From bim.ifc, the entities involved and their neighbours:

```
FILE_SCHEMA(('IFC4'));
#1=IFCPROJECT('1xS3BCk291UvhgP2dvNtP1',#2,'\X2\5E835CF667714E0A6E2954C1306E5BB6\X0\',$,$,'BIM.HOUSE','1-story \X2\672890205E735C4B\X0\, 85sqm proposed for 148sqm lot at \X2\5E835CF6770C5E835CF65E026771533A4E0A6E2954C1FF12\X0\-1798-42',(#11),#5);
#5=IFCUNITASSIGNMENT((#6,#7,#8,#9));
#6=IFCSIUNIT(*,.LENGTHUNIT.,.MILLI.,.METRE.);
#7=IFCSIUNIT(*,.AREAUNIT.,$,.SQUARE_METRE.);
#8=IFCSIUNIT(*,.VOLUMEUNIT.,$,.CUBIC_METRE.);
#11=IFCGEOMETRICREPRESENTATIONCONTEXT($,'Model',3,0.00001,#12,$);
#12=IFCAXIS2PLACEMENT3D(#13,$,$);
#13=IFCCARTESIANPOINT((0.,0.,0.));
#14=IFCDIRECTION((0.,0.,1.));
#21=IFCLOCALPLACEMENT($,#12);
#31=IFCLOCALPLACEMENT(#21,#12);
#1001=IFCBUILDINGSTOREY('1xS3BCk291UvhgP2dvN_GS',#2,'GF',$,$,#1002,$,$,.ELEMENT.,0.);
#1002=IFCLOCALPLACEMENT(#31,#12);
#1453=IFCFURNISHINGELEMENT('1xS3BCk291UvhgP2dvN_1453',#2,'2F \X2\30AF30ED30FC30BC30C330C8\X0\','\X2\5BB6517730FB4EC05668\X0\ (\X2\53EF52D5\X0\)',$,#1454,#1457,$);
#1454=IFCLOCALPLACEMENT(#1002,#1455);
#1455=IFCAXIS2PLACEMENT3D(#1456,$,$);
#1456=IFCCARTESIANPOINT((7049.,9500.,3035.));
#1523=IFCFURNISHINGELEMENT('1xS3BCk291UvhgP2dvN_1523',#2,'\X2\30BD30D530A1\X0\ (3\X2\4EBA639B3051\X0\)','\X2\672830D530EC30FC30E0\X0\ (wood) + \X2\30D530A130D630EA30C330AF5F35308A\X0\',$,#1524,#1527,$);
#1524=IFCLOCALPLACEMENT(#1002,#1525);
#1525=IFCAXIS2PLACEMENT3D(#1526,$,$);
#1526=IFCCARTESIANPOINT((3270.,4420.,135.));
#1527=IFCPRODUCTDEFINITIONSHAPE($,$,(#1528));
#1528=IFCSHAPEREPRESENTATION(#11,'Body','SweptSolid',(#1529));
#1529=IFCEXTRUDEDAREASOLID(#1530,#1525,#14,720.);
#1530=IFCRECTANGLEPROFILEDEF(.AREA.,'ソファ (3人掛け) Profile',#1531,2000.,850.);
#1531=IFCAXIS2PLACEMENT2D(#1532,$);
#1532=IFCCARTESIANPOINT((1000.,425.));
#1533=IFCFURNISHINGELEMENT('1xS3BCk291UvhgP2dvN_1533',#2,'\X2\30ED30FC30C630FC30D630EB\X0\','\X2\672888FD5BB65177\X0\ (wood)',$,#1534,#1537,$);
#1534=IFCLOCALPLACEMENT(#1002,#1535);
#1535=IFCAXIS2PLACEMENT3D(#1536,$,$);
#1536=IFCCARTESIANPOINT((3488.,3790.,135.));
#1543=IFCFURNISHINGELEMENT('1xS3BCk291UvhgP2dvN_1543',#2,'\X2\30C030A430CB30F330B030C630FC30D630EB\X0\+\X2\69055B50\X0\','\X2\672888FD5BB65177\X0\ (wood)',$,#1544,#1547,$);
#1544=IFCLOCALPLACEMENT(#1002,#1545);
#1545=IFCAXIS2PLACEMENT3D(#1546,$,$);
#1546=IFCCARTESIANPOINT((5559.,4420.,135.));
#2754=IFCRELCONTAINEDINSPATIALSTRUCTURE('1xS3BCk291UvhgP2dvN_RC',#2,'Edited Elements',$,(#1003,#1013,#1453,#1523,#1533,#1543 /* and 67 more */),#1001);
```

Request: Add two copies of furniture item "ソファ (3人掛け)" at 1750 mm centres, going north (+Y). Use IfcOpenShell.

```python
import numpy as np
import ifcopenshell
import ifcopenshell.api.geometry
import ifcopenshell.api.root
import ifcopenshell.util.element
import ifcopenshell.util.placement

model = ifcopenshell.open("bim.ifc")


def reuse_history(source, copy):
    """copy_class also copies each property set's owner history, people and application; keep the originals."""
    for rel in copy.IsDefinedBy:
        if rel.is_a("IfcRelDefinesByProperties") and (history := rel.RelatingPropertyDefinition.OwnerHistory):
            rel.RelatingPropertyDefinition.OwnerHistory = source.OwnerHistory
            ifcopenshell.util.element.remove_deep2(model, history)


source = model.by_guid("1xS3BCk291UvhgP2dvN_1523")
base = ifcopenshell.util.placement.get_local_placement(source.ObjectPlacement)
step = np.array([0.0, 1.0, 0.0]) * 1750.0

for i in range(1, 3):
    copy = ifcopenshell.api.root.copy_class(model, product=source)
    copy.Representation = ifcopenshell.util.element.copy_deep(
        model, source.Representation, exclude=["IfcGeometricRepresentationContext", "IfcRepresentationMap"]
    )
    reuse_history(source, copy)
    matrix = base.copy()
    matrix[:3, 3] += i * step
    print("added at", matrix[:3, 3].round(3) + 0.0)
    ifcopenshell.api.geometry.edit_object_placement(model, product=copy, matrix=matrix, is_si=False)

model.write("bim_v2.ifc")
```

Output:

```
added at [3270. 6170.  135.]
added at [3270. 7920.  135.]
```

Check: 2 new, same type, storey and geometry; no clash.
